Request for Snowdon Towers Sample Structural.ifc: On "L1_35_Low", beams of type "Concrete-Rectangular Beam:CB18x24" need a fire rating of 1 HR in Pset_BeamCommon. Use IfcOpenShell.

First a look at what the model holds.

```python
import ifcopenshell
import ifcopenshell.util.element

model = ifcopenshell.open("Snowdon Towers Sample Structural.ifc")
print(model.schema)
storey = next(s for s in model.by_type("IfcBuildingStorey") if s.Name == "L1_35_Low")
beams = [e for e in ifcopenshell.util.element.get_decomposition(storey) if e.is_a("IfcBeam")]
seen = {}
for e in beams:
    element_type = ifcopenshell.util.element.get_type(e)
    key = (element_type.Name if element_type != e and element_type else None, ifcopenshell.util.element.get_pset(e, "Pset_BeamCommon", "FireRating"))
    seen[key] = seen.get(key, 0) + 1
for (name, value), count in sorted(seen.items(), key=str):
    print(count, "x", name, "|", value)
```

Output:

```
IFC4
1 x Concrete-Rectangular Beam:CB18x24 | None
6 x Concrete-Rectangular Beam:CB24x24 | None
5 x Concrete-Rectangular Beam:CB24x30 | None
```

```python
import ifcopenshell
import ifcopenshell.api.pset
import ifcopenshell.util.element

model = ifcopenshell.open("Snowdon Towers Sample Structural.ifc")

storey = next(s for s in model.by_type("IfcBuildingStorey") if s.Name == "L1_35_Low")
beams = [e for e in ifcopenshell.util.element.get_decomposition(storey) if e.is_a("IfcBeam")]

count = 0
for e in beams:
    element_type = ifcopenshell.util.element.get_type(e)
    if element_type in (None, e) or element_type.Name != "Concrete-Rectangular Beam:CB18x24":
        continue
    # add_pset returns the element's existing set when there is one.
    pset = ifcopenshell.api.pset.add_pset(model, product=e, name="Pset_BeamCommon")
    ifcopenshell.api.pset.edit_pset(model, pset=pset, properties={"FireRating": "1 HR"})
    count += 1

print(count, "beams updated")

model.write("Snowdon Towers Sample Structural-out.ifc")
```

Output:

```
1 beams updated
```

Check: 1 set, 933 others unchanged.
